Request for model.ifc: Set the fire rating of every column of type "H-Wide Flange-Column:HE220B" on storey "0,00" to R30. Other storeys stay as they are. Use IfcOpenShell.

First a look at what the model holds.

```python
import ifcopenshell
import ifcopenshell.util.element

model = ifcopenshell.open("model.ifc")
print(model.schema)
storey = next(s for s in model.by_type("IfcBuildingStorey") if s.Name == "0,00")
columns = [e for e in ifcopenshell.util.element.get_decomposition(storey) if e.is_a("IfcColumn")]
seen = {}
for e in columns:
    element_type = ifcopenshell.util.element.get_type(e)
    key = (element_type.Name if element_type != e and element_type else None, ifcopenshell.util.element.get_pset(e, "Pset_ColumnCommon", "FireRating"))
    seen[key] = seen.get(key, 0) + 1
for (name, value), count in sorted(seen.items(), key=str):
    print(count, "x", name, "|", value)
```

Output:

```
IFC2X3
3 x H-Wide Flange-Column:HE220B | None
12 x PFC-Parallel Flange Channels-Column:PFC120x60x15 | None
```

```python
import ifcopenshell
import ifcopenshell.api.pset
import ifcopenshell.util.element

model = ifcopenshell.open("model.ifc")

storey = next(s for s in model.by_type("IfcBuildingStorey") if s.Name == "0,00")
columns = [e for e in ifcopenshell.util.element.get_decomposition(storey) if e.is_a("IfcColumn")]

count = 0
for e in columns:
    element_type = ifcopenshell.util.element.get_type(e)
    if element_type in (None, e) or element_type.Name != "H-Wide Flange-Column:HE220B":
        continue
    # add_pset returns the element's existing set when there is one.
    pset = ifcopenshell.api.pset.add_pset(model, product=e, name="Pset_ColumnCommon")
    ifcopenshell.api.pset.edit_pset(model, pset=pset, properties={"FireRating": "R30"})
    count += 1

print(count, "columns updated")

model.write("model_rev.ifc")
```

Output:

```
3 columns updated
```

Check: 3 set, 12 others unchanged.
